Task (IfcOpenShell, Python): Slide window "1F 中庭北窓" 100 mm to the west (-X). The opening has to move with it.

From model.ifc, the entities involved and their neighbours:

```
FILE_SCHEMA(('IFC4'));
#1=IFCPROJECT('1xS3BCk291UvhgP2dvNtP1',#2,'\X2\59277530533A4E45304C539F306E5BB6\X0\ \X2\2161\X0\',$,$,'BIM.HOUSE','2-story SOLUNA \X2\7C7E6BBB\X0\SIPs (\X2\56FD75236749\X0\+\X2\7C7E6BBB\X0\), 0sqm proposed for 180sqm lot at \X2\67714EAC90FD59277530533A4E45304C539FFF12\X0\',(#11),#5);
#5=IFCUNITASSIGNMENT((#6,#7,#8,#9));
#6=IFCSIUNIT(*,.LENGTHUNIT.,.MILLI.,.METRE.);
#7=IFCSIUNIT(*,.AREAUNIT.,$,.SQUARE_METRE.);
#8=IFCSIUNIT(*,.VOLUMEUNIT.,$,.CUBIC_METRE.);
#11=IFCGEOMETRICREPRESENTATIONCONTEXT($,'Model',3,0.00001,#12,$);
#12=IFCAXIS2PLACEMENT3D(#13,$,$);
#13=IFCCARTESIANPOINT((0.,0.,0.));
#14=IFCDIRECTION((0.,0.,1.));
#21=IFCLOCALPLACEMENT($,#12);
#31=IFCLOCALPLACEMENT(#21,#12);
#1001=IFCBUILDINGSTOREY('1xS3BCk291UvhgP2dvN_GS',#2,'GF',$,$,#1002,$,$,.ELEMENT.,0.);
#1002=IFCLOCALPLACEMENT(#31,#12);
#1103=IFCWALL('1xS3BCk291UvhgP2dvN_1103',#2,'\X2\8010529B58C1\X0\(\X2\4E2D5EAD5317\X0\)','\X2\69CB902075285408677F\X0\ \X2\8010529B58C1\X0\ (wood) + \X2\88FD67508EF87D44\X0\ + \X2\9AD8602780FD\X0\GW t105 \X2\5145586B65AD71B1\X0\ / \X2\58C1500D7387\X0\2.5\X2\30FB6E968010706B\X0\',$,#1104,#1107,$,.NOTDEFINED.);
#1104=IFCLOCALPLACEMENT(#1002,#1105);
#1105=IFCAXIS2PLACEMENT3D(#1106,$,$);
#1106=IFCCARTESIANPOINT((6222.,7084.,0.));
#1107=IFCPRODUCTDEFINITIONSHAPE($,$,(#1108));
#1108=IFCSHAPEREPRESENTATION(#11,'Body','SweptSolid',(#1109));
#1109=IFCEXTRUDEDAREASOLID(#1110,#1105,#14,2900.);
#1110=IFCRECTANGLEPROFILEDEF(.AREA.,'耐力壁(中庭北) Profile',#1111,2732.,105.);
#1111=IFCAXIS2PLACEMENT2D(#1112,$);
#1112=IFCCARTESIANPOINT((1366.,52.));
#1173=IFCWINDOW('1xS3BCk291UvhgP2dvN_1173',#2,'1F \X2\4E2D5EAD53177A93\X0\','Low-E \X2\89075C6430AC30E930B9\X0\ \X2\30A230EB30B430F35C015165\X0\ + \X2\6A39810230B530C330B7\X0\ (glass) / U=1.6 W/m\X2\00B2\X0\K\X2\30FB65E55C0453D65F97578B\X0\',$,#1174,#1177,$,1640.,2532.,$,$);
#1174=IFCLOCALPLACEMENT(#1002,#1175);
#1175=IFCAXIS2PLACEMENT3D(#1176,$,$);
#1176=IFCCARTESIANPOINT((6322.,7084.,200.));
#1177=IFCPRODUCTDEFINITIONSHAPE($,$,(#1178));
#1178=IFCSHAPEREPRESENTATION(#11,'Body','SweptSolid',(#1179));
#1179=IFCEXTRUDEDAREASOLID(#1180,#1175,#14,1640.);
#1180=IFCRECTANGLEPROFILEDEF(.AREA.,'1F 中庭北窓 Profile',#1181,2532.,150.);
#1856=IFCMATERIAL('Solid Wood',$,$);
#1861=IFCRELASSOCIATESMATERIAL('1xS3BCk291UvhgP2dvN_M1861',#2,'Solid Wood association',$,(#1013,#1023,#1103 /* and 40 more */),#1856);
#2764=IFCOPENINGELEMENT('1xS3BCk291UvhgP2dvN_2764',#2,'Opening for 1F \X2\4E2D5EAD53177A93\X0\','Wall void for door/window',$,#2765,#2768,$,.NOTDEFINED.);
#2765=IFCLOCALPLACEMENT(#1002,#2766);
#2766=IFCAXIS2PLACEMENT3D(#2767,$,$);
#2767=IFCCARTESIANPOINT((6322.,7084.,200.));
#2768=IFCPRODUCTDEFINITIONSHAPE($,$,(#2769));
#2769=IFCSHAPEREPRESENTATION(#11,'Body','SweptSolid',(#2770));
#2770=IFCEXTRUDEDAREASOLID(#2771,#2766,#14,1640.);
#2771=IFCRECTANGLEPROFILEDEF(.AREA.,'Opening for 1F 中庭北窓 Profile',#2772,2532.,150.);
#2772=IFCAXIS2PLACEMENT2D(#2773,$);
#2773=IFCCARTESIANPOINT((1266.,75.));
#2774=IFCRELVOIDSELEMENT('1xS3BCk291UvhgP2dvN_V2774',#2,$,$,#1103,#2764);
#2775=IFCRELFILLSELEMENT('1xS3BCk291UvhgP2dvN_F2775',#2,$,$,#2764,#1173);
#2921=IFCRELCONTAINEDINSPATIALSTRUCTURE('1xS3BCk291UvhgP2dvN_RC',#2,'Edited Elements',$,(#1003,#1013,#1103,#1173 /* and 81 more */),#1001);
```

```python
import ifcopenshell
import ifcopenshell.api.geometry
import ifcopenshell.util.placement
import ifcopenshell.util.unit

model = ifcopenshell.open("model.ifc")
unit_scale = ifcopenshell.util.unit.calculate_unit_scale(model)

window = model.by_id(1173)
opening = window.FillsVoids[0].RelatingOpeningElement
wall = opening.VoidsElements[0].RelatingBuildingElement

wall_matrix = ifcopenshell.util.placement.get_local_placement(wall.ObjectPlacement)
shift = wall_matrix[:3, 0] * -0.1 / unit_scale
before = ifcopenshell.util.placement.get_local_placement(window.ObjectPlacement)[:3, 3].copy()

# The window is not placed relative to its opening, so move both.
for product in (opening, window):
    matrix = ifcopenshell.util.placement.get_local_placement(product.ObjectPlacement)
    matrix[:3, 3] += shift
    ifcopenshell.api.geometry.edit_object_placement(model, product=product, matrix=matrix, is_si=False)

after = ifcopenshell.util.placement.get_local_placement(window.ObjectPlacement)[:3, 3]
print("window moved by", (after - before).round(3) + 0.0)

model.write("model_edited.ifc")
```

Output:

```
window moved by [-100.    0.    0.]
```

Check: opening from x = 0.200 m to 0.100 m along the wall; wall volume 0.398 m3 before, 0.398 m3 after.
